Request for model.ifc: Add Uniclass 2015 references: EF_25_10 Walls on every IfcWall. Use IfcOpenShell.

First a look at what the model holds.

```python
import ifcopenshell

model = ifcopenshell.open("model.ifc")
print(model.schema)
print("classifications:", [c.Name for c in model.by_type("IfcClassification")])
for ifc_class in ("IfcDoor", "IfcRoof", "IfcStair", "IfcWall", "IfcWindow"):
    print(ifc_class, len(model.by_type(ifc_class)))
```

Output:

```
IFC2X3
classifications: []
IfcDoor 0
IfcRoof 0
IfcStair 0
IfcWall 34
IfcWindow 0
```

```python
import ifcopenshell
import ifcopenshell.api.classification

model = ifcopenshell.open("model.ifc")

# IFC2X3 requires Source and Edition and has no link from the project to the system.
system = model.create_entity("IfcClassification", Source="NBS", Edition="2015", Name="Uniclass 2015")

codes = {
    "IfcWall": ("EF_25_10", "Walls"),
}
for ifc_class, (code, name) in codes.items():
    products = model.by_type(ifc_class)
    ifcopenshell.api.classification.add_reference(
        model, products=products, classification=system, identification=code, name=name
    )
    print(code, len(products))

model.write("model_rev.ifc")
```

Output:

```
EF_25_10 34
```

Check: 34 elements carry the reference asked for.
